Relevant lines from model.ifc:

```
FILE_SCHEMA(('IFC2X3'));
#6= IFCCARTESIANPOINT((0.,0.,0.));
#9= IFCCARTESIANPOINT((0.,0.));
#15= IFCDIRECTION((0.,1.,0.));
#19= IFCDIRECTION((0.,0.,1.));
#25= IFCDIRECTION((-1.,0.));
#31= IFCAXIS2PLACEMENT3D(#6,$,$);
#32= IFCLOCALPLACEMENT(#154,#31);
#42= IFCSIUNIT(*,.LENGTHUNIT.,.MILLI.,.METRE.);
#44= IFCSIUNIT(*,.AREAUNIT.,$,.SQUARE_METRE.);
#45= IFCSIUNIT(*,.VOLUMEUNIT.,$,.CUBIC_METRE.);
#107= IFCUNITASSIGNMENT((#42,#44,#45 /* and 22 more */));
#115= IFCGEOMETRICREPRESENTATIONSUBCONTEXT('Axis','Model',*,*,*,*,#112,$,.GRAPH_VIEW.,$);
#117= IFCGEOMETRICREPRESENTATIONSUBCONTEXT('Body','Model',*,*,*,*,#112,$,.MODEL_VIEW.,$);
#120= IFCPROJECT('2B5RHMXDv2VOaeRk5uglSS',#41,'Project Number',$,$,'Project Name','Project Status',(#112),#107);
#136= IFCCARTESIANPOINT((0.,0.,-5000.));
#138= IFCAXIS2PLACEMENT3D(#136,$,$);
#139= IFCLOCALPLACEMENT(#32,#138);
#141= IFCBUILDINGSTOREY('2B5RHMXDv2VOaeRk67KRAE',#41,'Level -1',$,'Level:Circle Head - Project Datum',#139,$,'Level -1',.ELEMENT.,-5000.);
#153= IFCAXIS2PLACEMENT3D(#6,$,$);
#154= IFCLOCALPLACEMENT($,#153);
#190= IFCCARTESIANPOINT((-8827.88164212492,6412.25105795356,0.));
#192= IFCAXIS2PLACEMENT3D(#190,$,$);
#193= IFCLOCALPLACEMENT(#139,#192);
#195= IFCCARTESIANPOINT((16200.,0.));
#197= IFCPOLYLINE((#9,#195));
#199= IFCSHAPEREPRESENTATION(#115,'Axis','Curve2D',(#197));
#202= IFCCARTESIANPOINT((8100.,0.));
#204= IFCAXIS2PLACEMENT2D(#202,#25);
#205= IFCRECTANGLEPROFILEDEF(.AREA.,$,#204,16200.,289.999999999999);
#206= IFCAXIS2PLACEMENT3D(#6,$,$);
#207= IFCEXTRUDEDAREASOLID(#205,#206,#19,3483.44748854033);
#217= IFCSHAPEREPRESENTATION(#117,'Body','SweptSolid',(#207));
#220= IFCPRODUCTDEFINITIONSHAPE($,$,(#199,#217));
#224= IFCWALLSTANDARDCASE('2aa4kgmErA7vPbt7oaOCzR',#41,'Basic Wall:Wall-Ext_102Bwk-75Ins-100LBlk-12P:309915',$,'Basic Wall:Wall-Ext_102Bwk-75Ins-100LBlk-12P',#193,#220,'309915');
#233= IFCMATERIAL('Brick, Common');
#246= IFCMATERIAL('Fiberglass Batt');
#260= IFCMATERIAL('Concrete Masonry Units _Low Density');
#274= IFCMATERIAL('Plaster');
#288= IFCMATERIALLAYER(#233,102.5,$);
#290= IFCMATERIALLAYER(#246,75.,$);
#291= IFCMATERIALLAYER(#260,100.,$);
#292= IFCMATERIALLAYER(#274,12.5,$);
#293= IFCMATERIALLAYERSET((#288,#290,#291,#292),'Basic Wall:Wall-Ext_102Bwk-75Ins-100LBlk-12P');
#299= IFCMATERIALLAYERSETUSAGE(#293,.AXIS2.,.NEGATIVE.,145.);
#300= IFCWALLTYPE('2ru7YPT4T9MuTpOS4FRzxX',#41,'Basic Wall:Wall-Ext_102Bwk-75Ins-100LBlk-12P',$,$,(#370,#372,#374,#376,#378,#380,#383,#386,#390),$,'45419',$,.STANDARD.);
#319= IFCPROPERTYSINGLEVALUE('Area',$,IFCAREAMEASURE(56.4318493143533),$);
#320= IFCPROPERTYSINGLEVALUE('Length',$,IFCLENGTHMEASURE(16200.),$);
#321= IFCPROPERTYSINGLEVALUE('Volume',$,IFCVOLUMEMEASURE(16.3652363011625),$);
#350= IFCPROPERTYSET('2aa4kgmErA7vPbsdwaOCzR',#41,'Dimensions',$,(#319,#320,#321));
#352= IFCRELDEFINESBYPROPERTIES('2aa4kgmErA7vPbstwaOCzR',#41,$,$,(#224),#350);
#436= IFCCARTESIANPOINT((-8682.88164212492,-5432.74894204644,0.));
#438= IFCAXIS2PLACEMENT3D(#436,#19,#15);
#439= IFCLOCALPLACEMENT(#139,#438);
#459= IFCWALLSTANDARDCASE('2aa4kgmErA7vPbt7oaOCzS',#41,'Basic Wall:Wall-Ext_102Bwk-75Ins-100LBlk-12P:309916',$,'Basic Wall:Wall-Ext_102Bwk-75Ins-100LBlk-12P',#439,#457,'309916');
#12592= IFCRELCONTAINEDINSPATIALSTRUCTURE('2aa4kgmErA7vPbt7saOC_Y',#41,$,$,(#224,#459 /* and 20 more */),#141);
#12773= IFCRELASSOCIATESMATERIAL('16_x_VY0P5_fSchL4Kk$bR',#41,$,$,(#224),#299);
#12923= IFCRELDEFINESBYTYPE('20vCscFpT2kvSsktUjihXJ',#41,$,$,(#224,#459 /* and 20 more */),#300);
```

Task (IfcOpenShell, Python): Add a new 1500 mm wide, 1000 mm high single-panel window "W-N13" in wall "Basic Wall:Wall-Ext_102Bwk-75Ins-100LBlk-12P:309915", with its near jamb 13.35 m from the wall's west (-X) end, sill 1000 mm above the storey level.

```python
import numpy as np
import ifcopenshell
import ifcopenshell.api.feature
import ifcopenshell.api.geometry
import ifcopenshell.api.pset
import ifcopenshell.api.root
import ifcopenshell.api.spatial
import ifcopenshell.api.type
import ifcopenshell.geom
import ifcopenshell.util.element
import ifcopenshell.util.placement
import ifcopenshell.util.representation
import ifcopenshell.util.shape
import ifcopenshell.util.unit

model = ifcopenshell.open("model.ifc")
unit_scale = ifcopenshell.util.unit.calculate_unit_scale(model)
area_scale = ifcopenshell.util.unit.calculate_unit_scale(model, "AREAUNIT")
volume_scale = ifcopenshell.util.unit.calculate_unit_scale(model, "VOLUMEUNIT")
settings = ifcopenshell.geom.settings()


def volume(element):
    """Net volume in cubic metres, openings subtracted."""
    shape = ifcopenshell.geom.create_shape(settings, element)
    return ifcopenshell.util.shape.get_volume(shape.geometry)


wall = model.by_guid("2aa4kgmErA7vPbt7oaOCzR")
storey = ifcopenshell.util.element.get_container(wall, ifc_class="IfcBuildingStorey")
context = ifcopenshell.util.representation.get_context(model, "Model", "Body", "MODEL_VIEW")
before = volume(wall)

width, height, from_end, sill = 1.5, 1, 13.35, 1  # metres

# The wall runs along its own X axis, and the end named is its -X end.
wall_shape = ifcopenshell.geom.create_shape(settings, wall)
x, y, z = ifcopenshell.util.shape.get_vertices(wall_shape.geometry).T
start = x.min() + from_end
face, thickness = float(y.min()), float(y.max() - y.min())
wall_matrix = ifcopenshell.util.placement.get_local_placement(wall.ObjectPlacement)
level = ifcopenshell.util.placement.get_local_placement(storey.ObjectPlacement)[2, 3]


def in_wall(x, y):
    """Placement at x, y metres in the wall's axes, at sill height."""
    matrix = wall_matrix.copy()
    matrix[:, 3] = wall_matrix @ np.array([x / unit_scale, y / unit_scale, 0.0, 1.0])
    matrix[2, 3] = level + sill / unit_scale
    return matrix


# Opening: a box that overshoots both wall faces by 50 mm.
opening = ifcopenshell.api.root.create_entity(model, ifc_class="IfcOpeningElement")
box = ifcopenshell.api.geometry.add_wall_representation(
    model, context=context, length=width, height=height, thickness=thickness + 0.1
)
ifcopenshell.api.geometry.assign_representation(model, product=opening, representation=box)
ifcopenshell.api.geometry.edit_object_placement(model, product=opening, matrix=in_wall(start, face - 0.05), is_si=False)
ifcopenshell.api.feature.add_feature(model, feature=opening, element=wall)

window = ifcopenshell.api.root.create_entity(model, ifc_class="IfcWindow", name="W-N13")
window.OverallWidth, window.OverallHeight = width / unit_scale, height / unit_scale
body = ifcopenshell.api.geometry.add_window_representation(
    model,
    context=context,
    overall_width=window.OverallWidth,
    overall_height=window.OverallHeight,
    partition_type="SINGLE_PANEL",
)
ifcopenshell.api.geometry.assign_representation(model, product=window, representation=body)
ifcopenshell.api.spatial.assign_container(model, products=[window], relating_structure=storey)
fills = ifcopenshell.api.feature.add_filling(model, opening=opening, element=window)
fills.OwnerHistory = window.OwnerHistory  # required in IFC2X3

# IFC2X3 keeps the operation on the window style.
style = ifcopenshell.api.root.create_entity(model, ifc_class="IfcWindowStyle", name="W-N13")
style.OperationType, style.ConstructionType = "SINGLE_PANEL", "NOTDEFINED"
style.ParameterTakesPrecedence = style.Sizeable = False
ifcopenshell.api.type.assign_type(model, related_objects=[window], relating_type=style)

# Centre the window in the wall's thickness.
ifcopenshell.api.geometry.edit_object_placement(model, product=window, matrix=in_wall(start, face), is_si=False)
window_shape = ifcopenshell.geom.create_shape(settings, window)
depth = ifcopenshell.util.shape.get_vertices(window_shape.geometry)[:, 1]
offset = face + thickness / 2 - (depth.min() + depth.max()) / 2
ifcopenshell.api.geometry.edit_object_placement(model, product=window, matrix=in_wall(start, offset), is_si=False)

after = volume(wall)

# Update the wall's stored quantities.
pset = model.by_id(ifcopenshell.util.element.get_pset(wall, "Dimensions", should_inherit=False)["id"])
ifcopenshell.api.pset.edit_pset(model, pset=pset, properties={
    "Area": model.create_entity("IfcAreaMeasure", after / thickness / area_scale),
    "Volume": model.create_entity("IfcVolumeMeasure", after / volume_scale),
})

print(f"wall volume {before:.3f} -> {after:.3f} m3")

model.write("model-out.ifc")
```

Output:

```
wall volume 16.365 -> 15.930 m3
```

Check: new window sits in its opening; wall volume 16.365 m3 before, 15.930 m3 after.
